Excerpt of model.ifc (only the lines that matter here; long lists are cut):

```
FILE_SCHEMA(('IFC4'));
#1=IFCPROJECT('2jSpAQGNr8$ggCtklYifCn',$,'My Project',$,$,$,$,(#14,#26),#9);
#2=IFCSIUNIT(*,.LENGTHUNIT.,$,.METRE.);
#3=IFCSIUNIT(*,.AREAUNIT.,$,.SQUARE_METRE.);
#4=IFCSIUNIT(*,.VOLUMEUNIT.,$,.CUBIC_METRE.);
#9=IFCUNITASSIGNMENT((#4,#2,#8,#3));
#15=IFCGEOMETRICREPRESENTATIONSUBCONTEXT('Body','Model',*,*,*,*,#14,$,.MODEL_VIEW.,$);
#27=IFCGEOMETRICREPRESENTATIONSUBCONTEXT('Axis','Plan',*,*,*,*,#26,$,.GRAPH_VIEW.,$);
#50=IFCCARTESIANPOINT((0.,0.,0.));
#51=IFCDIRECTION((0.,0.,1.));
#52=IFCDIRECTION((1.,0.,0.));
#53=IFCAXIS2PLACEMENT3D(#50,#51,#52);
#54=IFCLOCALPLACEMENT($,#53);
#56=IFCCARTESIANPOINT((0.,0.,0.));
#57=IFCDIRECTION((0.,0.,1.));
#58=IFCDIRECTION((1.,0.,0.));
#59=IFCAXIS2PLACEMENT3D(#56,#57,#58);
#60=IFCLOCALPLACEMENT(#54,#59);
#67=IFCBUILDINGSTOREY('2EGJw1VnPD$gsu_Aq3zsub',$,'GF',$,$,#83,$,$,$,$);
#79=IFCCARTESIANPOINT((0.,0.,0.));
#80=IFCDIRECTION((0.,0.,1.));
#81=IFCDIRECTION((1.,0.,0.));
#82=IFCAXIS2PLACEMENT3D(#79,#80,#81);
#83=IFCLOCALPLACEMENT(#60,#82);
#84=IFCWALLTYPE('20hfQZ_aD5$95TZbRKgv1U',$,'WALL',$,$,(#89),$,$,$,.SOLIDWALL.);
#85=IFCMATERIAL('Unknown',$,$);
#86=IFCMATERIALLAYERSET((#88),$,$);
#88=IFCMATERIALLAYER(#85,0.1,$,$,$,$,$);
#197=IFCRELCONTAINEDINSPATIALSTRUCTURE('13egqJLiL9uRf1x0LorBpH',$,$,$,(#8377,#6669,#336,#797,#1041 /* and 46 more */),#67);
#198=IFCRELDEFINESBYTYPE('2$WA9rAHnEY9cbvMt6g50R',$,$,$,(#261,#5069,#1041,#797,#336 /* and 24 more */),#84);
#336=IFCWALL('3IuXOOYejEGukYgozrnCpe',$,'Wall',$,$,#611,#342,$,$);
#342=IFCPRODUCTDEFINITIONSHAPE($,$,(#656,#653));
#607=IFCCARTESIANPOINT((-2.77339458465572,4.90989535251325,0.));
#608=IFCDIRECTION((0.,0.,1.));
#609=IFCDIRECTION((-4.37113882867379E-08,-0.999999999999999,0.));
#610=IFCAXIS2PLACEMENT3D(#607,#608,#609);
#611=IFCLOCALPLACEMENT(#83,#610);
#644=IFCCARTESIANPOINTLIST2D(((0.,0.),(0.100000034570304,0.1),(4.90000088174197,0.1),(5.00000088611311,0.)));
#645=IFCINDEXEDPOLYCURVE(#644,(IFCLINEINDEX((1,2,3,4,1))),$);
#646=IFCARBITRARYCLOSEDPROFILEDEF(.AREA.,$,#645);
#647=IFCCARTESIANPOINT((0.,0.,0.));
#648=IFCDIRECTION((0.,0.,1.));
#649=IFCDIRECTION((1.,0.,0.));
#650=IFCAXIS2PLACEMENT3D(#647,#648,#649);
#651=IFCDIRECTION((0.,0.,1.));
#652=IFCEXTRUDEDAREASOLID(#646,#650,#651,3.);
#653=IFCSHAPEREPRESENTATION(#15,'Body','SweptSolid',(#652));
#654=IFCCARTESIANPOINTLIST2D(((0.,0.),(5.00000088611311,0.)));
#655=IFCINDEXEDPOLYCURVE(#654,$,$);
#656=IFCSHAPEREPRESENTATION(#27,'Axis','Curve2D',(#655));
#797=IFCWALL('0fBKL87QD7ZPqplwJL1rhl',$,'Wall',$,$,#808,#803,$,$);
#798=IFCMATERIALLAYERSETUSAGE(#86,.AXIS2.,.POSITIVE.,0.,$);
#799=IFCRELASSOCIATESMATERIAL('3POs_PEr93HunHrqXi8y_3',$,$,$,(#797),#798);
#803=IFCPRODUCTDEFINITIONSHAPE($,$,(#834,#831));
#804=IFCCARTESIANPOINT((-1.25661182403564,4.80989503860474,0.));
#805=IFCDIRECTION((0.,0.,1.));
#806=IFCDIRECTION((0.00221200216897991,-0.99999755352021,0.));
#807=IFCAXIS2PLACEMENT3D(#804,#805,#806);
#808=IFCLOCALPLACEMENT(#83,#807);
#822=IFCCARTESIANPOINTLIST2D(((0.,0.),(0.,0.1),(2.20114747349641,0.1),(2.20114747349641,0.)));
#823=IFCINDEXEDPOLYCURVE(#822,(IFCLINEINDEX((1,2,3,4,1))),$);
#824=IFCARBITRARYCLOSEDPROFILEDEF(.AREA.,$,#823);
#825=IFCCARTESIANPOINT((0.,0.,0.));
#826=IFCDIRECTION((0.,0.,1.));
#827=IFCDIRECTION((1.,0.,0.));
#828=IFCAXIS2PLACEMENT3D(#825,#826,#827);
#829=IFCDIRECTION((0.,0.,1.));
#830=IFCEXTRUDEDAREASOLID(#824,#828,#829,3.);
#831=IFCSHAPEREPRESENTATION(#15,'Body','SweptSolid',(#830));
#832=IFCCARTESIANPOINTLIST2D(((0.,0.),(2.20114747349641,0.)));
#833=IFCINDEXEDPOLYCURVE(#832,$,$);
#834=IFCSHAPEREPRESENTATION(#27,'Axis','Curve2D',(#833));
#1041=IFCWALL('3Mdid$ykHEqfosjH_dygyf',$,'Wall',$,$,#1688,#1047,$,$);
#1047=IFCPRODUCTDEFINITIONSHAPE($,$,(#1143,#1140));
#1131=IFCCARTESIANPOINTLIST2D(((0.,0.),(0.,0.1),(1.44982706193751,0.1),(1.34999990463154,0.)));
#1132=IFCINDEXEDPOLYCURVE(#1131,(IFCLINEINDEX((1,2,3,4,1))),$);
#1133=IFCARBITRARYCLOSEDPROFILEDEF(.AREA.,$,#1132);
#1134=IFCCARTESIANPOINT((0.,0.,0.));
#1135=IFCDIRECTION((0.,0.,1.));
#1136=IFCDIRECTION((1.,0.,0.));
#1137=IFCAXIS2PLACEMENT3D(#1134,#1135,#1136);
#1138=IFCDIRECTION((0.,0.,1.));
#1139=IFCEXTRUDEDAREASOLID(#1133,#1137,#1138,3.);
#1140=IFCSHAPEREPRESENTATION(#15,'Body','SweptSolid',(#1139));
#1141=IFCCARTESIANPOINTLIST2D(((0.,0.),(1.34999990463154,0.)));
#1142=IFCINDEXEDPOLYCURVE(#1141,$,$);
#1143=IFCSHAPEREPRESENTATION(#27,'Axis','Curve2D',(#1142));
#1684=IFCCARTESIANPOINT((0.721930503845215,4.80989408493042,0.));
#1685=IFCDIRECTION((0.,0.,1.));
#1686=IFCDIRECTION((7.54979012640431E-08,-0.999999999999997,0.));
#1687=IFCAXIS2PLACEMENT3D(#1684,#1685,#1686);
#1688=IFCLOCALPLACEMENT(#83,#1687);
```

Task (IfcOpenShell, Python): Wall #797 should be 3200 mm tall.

```python
import ifcopenshell
import ifcopenshell.geom
import ifcopenshell.util.representation
import ifcopenshell.util.shape
import ifcopenshell.util.unit

model = ifcopenshell.open("model.ifc")
unit_scale = ifcopenshell.util.unit.calculate_unit_scale(model)
settings = ifcopenshell.geom.settings()


def volume(element):
    """Net volume in cubic metres, openings subtracted."""
    shape = ifcopenshell.geom.create_shape(settings, element)
    return ifcopenshell.util.shape.get_volume(shape.geometry)


wall = model.by_id(797)
before = volume(wall)

body = ifcopenshell.util.representation.get_representation(wall, "Model", "Body")
solid = body.Items[0]
old_height = solid.Depth
solid.Depth = 3.2 / unit_scale
after = volume(wall)

print(f"height {old_height:g} -> {solid.Depth:g}, volume {before:.3f} -> {after:.3f} m3")

model.write("model-out.ifc")
```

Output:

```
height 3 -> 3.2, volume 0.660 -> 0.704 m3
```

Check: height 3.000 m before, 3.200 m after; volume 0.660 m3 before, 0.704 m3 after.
